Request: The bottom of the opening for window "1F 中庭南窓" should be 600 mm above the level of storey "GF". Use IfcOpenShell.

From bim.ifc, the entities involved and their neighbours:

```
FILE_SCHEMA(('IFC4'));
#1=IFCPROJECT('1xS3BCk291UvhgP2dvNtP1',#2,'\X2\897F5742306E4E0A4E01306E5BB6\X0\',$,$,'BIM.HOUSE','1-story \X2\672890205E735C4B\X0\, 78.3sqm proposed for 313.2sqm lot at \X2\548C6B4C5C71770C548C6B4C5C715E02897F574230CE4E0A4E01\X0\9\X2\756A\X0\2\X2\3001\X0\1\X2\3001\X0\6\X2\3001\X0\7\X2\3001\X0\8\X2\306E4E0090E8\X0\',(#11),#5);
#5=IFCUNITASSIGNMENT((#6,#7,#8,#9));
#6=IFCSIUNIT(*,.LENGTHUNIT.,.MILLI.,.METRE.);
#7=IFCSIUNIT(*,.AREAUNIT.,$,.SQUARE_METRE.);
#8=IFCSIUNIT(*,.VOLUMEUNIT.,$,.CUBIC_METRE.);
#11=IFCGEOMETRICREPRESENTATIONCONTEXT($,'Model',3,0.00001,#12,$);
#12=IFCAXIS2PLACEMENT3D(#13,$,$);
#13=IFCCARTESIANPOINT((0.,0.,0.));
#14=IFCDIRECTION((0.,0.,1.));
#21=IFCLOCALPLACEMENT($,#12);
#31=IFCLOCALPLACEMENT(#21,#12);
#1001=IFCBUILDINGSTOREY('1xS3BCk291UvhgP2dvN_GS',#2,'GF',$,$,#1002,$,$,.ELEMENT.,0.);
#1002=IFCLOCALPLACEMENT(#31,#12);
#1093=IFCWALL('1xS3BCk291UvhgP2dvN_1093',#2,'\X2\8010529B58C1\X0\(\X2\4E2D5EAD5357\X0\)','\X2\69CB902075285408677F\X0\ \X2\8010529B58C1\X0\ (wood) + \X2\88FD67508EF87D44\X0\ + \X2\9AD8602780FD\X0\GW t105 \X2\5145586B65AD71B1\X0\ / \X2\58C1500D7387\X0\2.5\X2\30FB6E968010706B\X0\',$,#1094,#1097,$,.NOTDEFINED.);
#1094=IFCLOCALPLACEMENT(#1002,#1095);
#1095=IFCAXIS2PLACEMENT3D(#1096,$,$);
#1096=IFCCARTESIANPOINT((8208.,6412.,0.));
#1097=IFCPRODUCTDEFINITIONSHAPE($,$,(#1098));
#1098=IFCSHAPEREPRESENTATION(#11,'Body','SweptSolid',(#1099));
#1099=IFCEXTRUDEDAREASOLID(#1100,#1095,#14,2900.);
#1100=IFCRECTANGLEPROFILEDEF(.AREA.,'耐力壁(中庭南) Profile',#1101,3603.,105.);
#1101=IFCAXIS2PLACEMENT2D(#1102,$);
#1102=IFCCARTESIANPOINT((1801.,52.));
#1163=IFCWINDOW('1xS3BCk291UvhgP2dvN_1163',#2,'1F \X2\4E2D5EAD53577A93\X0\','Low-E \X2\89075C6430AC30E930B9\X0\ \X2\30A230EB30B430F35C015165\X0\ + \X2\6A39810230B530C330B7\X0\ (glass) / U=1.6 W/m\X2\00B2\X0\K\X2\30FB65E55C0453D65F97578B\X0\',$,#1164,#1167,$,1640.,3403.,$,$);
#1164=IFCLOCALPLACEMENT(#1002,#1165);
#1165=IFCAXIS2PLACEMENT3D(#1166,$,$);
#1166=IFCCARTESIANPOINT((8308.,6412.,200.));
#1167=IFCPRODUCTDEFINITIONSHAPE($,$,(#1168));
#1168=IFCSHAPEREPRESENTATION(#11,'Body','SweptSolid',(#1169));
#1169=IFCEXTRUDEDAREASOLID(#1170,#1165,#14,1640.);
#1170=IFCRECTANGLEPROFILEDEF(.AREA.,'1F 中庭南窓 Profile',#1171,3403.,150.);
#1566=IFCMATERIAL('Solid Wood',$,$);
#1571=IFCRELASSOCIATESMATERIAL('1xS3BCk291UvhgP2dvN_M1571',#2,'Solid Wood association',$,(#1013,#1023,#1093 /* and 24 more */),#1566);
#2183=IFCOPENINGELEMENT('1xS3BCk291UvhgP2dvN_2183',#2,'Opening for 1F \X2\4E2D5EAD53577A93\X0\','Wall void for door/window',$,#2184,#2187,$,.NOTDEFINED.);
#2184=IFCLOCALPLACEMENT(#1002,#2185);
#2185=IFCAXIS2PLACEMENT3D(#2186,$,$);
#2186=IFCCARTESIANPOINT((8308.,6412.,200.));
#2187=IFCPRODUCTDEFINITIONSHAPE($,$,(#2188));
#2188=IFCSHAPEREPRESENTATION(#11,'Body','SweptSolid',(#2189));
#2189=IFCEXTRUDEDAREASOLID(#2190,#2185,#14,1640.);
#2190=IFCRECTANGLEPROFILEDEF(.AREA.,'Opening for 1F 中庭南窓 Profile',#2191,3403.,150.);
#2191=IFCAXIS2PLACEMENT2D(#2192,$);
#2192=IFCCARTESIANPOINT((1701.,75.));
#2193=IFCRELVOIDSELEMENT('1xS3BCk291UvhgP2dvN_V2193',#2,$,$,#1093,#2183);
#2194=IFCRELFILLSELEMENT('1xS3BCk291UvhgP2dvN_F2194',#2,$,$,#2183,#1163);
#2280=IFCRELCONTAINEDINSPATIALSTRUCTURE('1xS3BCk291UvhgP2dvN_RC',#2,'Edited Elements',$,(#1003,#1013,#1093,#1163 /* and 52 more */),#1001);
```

```python
import numpy as np
import ifcopenshell
import ifcopenshell.api.geometry
import ifcopenshell.geom
import ifcopenshell.util.element
import ifcopenshell.util.placement
import ifcopenshell.util.shape
import ifcopenshell.util.unit

model = ifcopenshell.open("bim.ifc")
unit_scale = ifcopenshell.util.unit.calculate_unit_scale(model)

window = model.by_guid("1xS3BCk291UvhgP2dvN_1163")
opening = window.FillsVoids[0].RelatingOpeningElement
storey = ifcopenshell.util.element.get_container(window, ifc_class="IfcBuildingStorey")
level = ifcopenshell.util.placement.get_local_placement(storey.ObjectPlacement)[2, 3]

# The opening's origin need not be at the sill, so measure its lowest point.
shape = ifcopenshell.geom.create_shape(ifcopenshell.geom.settings(), opening)
bottom = ifcopenshell.util.shape.get_shape_bottom_elevation(shape, shape.geometry) / unit_scale
dz = level + 0.6 / unit_scale - bottom

shift = np.array([0.0, 0.0, dz])
# The window is not placed relative to its opening, so move both.
for product in (opening, window):
    matrix = ifcopenshell.util.placement.get_local_placement(product.ObjectPlacement)
    matrix[:3, 3] += shift
    ifcopenshell.api.geometry.edit_object_placement(model, product=product, matrix=matrix, is_si=False)

print(f"moved by {dz * unit_scale:+.3f} m")

model.write("bim_v2.ifc")
```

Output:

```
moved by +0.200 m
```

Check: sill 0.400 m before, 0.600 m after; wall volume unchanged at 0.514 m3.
